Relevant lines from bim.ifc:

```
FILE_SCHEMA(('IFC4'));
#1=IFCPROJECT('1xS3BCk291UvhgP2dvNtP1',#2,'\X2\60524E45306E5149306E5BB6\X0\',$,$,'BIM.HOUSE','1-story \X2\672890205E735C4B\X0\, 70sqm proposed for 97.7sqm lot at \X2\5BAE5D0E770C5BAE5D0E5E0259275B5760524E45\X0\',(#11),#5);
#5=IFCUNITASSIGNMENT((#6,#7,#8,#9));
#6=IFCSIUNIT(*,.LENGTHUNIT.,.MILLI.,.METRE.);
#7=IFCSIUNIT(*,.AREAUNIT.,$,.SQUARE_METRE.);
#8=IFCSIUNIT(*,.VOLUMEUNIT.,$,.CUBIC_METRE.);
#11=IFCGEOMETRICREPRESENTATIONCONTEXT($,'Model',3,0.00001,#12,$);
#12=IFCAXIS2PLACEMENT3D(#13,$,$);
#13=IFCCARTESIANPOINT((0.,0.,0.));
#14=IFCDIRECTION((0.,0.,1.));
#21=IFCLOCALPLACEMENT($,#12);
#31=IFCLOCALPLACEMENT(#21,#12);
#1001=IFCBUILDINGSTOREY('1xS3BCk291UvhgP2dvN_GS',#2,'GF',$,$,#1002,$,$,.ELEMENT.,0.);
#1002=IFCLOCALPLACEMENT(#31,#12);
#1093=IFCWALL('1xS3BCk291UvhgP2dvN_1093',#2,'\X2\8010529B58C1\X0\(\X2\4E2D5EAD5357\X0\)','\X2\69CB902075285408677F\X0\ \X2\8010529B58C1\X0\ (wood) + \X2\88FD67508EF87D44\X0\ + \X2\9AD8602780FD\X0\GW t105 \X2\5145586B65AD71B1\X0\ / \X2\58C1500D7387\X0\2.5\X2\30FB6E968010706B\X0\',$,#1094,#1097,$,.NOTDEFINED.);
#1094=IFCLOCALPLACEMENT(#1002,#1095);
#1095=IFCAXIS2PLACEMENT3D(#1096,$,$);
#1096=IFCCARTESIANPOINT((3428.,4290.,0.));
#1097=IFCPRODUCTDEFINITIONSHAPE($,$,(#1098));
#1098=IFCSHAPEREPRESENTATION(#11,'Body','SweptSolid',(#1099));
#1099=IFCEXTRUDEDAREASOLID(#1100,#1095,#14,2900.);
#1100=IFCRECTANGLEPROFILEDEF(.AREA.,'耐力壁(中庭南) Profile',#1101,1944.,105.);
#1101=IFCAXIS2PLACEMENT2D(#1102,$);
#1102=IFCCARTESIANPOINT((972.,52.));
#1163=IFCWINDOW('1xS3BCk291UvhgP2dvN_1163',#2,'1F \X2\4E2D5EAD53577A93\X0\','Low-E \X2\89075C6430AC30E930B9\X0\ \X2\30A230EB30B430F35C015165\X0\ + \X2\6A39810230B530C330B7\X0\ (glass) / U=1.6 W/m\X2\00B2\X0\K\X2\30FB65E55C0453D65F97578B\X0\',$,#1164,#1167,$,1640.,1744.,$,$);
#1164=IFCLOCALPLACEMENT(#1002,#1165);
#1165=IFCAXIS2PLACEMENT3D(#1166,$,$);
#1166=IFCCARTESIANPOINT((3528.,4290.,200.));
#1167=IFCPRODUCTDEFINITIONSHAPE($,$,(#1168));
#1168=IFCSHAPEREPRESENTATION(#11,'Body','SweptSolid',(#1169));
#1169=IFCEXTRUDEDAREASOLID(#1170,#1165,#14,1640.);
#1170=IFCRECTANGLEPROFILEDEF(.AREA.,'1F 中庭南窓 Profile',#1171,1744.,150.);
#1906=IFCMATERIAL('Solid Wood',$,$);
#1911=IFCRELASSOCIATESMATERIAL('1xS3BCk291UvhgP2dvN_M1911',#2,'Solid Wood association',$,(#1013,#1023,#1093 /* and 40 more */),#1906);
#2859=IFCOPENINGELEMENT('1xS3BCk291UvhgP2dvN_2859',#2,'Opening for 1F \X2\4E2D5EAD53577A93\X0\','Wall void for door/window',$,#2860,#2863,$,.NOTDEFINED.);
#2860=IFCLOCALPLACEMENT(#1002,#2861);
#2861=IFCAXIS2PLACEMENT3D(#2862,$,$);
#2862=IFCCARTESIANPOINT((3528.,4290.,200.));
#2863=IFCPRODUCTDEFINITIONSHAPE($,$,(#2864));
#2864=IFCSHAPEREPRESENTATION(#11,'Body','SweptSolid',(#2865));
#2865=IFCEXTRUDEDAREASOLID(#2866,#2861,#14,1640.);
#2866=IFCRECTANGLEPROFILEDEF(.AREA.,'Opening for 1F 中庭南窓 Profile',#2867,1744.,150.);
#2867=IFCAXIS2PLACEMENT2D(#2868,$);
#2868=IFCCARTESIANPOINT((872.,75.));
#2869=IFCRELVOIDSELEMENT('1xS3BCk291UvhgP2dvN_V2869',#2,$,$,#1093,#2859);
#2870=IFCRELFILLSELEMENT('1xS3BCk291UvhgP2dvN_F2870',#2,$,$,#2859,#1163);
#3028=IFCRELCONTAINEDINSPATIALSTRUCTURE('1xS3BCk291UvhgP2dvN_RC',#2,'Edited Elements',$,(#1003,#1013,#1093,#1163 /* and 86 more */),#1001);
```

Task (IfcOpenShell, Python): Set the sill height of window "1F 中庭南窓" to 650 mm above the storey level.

```python
import numpy as np
import ifcopenshell
import ifcopenshell.api.geometry
import ifcopenshell.geom
import ifcopenshell.util.element
import ifcopenshell.util.placement
import ifcopenshell.util.shape
import ifcopenshell.util.unit

model = ifcopenshell.open("bim.ifc")
unit_scale = ifcopenshell.util.unit.calculate_unit_scale(model)

window = model.by_guid("1xS3BCk291UvhgP2dvN_1163")
opening = window.FillsVoids[0].RelatingOpeningElement
storey = ifcopenshell.util.element.get_container(window, ifc_class="IfcBuildingStorey")
level = ifcopenshell.util.placement.get_local_placement(storey.ObjectPlacement)[2, 3]

# The opening's origin need not be at the sill, so measure its lowest point.
shape = ifcopenshell.geom.create_shape(ifcopenshell.geom.settings(), opening)
bottom = ifcopenshell.util.shape.get_shape_bottom_elevation(shape, shape.geometry) / unit_scale
dz = level + 0.65 / unit_scale - bottom

shift = np.array([0.0, 0.0, dz])
# The window is not placed relative to its opening, so move both.
for product in (opening, window):
    matrix = ifcopenshell.util.placement.get_local_placement(product.ObjectPlacement)
    matrix[:3, 3] += shift
    ifcopenshell.api.geometry.edit_object_placement(model, product=product, matrix=matrix, is_si=False)

print(f"moved by {dz * unit_scale:+.3f} m")

model.write("bim_v2.ifc")
```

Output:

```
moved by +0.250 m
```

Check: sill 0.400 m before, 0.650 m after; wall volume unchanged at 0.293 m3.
